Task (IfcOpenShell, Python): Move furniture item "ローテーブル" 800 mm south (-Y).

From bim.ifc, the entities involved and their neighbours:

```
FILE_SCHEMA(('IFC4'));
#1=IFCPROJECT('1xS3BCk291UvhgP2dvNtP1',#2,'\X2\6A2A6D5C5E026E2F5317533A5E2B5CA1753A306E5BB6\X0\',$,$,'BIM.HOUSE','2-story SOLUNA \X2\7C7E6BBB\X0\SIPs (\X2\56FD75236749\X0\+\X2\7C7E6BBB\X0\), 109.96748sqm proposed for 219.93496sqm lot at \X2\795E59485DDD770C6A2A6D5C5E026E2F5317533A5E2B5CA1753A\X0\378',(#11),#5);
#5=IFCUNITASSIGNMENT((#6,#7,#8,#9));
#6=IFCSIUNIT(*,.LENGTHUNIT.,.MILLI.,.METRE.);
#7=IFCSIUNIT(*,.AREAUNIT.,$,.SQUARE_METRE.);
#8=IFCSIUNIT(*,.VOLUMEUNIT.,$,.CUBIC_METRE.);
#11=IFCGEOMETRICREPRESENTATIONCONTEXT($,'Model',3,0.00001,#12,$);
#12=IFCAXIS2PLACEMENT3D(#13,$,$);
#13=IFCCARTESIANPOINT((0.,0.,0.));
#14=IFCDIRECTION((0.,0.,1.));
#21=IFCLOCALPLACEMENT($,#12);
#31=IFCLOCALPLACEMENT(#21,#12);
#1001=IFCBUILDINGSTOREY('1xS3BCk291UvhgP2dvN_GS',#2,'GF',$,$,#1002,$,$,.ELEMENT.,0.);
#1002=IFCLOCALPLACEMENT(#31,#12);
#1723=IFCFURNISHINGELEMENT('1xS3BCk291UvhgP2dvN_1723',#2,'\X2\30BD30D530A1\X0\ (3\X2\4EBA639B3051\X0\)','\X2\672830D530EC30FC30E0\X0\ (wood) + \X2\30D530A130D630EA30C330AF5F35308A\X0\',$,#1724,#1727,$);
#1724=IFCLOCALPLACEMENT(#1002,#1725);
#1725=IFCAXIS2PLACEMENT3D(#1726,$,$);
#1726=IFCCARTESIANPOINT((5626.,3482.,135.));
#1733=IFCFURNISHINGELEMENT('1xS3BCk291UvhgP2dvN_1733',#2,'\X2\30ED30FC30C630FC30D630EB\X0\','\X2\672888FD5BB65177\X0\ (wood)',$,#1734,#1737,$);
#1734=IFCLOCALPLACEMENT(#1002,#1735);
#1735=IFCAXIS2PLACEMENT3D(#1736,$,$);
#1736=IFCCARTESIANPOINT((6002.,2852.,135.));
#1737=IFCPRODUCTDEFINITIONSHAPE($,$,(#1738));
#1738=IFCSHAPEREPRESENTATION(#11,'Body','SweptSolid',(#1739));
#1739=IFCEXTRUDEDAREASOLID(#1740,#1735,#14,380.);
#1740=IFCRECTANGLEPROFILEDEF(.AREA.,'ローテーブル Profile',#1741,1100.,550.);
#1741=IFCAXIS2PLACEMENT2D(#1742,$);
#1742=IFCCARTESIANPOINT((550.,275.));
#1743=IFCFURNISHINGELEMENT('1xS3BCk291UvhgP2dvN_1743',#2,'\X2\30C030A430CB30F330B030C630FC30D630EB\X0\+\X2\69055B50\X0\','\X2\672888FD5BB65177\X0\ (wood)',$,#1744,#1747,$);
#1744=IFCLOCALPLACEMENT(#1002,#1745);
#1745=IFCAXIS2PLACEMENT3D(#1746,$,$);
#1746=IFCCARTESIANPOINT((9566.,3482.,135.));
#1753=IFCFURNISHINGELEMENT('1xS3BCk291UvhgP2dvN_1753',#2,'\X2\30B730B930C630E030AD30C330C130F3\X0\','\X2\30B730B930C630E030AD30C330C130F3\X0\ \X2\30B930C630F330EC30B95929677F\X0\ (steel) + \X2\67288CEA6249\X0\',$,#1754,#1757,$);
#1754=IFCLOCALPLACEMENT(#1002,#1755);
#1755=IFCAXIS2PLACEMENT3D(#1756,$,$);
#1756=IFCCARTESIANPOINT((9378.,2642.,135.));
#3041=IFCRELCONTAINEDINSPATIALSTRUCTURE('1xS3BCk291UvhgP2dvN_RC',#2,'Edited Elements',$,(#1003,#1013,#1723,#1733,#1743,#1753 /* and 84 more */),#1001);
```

```python
import ifcopenshell
import ifcopenshell.api.geometry
import ifcopenshell.util.placement

model = ifcopenshell.open("bim.ifc")

item = model.by_guid("1xS3BCk291UvhgP2dvN_1733")
matrix = ifcopenshell.util.placement.get_local_placement(item.ObjectPlacement)
matrix[1, 3] -= 800.0
ifcopenshell.api.geometry.edit_object_placement(model, product=item, matrix=matrix, is_si=False)

print(ifcopenshell.util.placement.get_local_placement(item.ObjectPlacement).round(3) + 0.0)

model.write("bim_rev.ifc")
```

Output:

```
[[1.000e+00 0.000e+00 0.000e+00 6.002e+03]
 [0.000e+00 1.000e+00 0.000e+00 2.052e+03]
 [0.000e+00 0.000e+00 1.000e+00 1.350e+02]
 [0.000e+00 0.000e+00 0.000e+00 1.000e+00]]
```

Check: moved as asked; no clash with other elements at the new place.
